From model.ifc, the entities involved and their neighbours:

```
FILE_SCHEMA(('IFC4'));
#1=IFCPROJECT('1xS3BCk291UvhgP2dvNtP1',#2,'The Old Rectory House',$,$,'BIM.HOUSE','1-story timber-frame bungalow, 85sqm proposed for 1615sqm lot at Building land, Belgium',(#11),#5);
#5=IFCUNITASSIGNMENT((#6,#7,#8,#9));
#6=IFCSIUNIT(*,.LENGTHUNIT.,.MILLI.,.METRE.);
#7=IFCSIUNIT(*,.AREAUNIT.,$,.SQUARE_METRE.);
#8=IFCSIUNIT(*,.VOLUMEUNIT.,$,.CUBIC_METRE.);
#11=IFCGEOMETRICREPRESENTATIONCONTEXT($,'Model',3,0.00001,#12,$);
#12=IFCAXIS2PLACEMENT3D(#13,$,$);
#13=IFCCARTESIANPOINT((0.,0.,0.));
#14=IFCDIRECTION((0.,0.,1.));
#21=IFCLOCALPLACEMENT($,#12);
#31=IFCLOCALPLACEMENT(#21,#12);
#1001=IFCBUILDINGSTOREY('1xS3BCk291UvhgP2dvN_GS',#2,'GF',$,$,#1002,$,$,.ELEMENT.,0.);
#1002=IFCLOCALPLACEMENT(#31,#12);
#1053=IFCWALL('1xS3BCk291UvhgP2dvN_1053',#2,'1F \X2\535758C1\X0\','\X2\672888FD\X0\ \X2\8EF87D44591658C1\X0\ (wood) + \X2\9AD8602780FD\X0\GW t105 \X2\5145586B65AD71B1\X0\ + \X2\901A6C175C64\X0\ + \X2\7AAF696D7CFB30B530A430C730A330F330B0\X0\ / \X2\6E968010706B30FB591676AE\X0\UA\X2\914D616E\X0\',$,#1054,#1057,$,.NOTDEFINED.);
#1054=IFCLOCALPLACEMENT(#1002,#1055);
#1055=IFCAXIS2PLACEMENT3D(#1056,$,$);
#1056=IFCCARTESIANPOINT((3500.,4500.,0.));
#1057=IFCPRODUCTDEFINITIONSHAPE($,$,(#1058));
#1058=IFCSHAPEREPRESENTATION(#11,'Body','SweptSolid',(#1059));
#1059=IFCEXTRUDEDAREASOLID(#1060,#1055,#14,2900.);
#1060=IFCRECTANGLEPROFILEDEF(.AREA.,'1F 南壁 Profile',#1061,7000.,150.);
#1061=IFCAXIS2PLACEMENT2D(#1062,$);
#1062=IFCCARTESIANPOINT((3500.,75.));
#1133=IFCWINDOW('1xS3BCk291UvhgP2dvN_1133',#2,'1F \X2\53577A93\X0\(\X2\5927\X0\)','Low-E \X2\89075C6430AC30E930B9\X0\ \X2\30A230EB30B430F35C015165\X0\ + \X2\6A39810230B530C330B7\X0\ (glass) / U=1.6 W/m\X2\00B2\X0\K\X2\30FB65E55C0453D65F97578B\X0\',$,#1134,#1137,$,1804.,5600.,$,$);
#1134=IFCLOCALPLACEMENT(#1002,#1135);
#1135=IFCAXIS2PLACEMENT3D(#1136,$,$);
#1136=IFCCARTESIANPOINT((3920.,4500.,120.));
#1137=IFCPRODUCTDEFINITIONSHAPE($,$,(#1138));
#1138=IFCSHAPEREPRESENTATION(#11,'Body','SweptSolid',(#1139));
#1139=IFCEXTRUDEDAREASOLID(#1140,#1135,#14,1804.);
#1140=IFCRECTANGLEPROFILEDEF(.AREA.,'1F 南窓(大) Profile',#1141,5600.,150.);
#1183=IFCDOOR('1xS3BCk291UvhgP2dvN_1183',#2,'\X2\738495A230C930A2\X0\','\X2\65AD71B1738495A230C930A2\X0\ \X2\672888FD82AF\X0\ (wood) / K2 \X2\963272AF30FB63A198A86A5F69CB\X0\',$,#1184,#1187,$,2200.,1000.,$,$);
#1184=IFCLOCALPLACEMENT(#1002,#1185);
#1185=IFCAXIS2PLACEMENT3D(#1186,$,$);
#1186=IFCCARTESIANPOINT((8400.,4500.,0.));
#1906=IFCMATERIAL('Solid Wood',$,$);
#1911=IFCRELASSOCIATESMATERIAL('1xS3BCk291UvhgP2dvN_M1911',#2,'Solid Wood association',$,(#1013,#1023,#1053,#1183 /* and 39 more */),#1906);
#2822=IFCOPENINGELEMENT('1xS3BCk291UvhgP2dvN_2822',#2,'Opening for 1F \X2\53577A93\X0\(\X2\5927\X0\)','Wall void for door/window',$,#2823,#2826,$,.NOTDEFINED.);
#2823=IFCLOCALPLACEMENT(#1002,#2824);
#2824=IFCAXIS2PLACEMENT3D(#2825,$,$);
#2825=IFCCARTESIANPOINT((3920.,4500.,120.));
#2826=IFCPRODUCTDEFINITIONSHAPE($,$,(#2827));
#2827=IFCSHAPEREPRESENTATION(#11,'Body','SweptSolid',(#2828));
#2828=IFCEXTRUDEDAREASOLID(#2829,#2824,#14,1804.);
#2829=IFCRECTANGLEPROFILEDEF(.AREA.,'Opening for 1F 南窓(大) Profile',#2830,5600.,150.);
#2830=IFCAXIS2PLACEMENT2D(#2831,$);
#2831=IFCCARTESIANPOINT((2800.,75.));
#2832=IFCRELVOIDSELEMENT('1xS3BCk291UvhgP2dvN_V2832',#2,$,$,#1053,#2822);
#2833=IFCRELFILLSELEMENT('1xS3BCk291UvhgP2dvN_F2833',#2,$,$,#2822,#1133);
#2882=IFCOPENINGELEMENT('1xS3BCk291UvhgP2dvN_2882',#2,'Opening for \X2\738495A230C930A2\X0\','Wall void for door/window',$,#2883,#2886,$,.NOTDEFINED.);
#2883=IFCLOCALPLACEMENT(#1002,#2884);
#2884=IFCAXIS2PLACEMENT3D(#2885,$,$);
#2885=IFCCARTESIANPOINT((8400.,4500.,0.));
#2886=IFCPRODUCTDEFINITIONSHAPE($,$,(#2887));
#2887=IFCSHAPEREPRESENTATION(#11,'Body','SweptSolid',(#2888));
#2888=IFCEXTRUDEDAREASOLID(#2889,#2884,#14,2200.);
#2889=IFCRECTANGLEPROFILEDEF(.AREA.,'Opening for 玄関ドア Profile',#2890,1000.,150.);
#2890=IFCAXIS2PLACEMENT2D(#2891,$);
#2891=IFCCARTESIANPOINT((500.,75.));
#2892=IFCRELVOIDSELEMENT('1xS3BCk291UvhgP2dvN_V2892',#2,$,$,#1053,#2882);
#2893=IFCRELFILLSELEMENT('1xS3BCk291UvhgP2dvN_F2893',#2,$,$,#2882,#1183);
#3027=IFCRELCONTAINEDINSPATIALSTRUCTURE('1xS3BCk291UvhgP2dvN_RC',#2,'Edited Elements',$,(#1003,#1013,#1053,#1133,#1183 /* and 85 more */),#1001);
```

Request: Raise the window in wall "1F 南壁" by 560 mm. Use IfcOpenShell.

```python
import numpy as np
import ifcopenshell
import ifcopenshell.api.geometry
import ifcopenshell.util.placement
import ifcopenshell.util.unit

model = ifcopenshell.open("model.ifc")
unit_scale = ifcopenshell.util.unit.calculate_unit_scale(model)

window = model.by_guid("1xS3BCk291UvhgP2dvN_1133")
opening = window.FillsVoids[0].RelatingOpeningElement
dz = 560.0

shift = np.array([0.0, 0.0, dz])
# The window is not placed relative to its opening, so move both.
for product in (opening, window):
    matrix = ifcopenshell.util.placement.get_local_placement(product.ObjectPlacement)
    matrix[:3, 3] += shift
    ifcopenshell.api.geometry.edit_object_placement(model, product=product, matrix=matrix, is_si=False)

print(f"moved by {dz * unit_scale:+.3f} m")

model.write("model_edited.ifc")
```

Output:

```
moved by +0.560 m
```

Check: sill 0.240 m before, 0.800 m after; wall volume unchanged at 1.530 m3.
